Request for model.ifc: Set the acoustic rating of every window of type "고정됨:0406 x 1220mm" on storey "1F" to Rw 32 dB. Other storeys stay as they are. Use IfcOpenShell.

First a look at what the model holds.

```python
import ifcopenshell
import ifcopenshell.util.element

model = ifcopenshell.open("model.ifc")
print(model.schema)
storey = next(s for s in model.by_type("IfcBuildingStorey") if s.Name == "1F")
windows = [e for e in ifcopenshell.util.element.get_decomposition(storey) if e.is_a("IfcWindow")]
seen = {}
for e in windows:
    element_type = ifcopenshell.util.element.get_type(e)
    key = (element_type.Name if element_type != e and element_type else None, ifcopenshell.util.element.get_pset(e, "Pset_WindowCommon", "AcousticRating"))
    seen[key] = seen.get(key, 0) + 1
for (name, value), count in sorted(seen.items(), key=str):
    print(count, "x", name, "|", value)
```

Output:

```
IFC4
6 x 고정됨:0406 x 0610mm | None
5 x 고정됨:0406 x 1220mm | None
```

```python
import ifcopenshell
import ifcopenshell.api.pset
import ifcopenshell.util.element

model = ifcopenshell.open("model.ifc")

storey = next(s for s in model.by_type("IfcBuildingStorey") if s.Name == "1F")
windows = [e for e in ifcopenshell.util.element.get_decomposition(storey) if e.is_a("IfcWindow")]

count = 0
for e in windows:
    element_type = ifcopenshell.util.element.get_type(e)
    if element_type in (None, e) or element_type.Name != "고정됨:0406 x 1220mm":
        continue
    # add_pset returns the element's existing set when there is one.
    pset = ifcopenshell.api.pset.add_pset(model, product=e, name="Pset_WindowCommon")
    ifcopenshell.api.pset.edit_pset(model, pset=pset, properties={"AcousticRating": "Rw 32 dB"})
    count += 1

print(count, "windows updated")

model.write("model_v2.ifc")
```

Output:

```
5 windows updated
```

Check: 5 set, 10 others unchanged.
